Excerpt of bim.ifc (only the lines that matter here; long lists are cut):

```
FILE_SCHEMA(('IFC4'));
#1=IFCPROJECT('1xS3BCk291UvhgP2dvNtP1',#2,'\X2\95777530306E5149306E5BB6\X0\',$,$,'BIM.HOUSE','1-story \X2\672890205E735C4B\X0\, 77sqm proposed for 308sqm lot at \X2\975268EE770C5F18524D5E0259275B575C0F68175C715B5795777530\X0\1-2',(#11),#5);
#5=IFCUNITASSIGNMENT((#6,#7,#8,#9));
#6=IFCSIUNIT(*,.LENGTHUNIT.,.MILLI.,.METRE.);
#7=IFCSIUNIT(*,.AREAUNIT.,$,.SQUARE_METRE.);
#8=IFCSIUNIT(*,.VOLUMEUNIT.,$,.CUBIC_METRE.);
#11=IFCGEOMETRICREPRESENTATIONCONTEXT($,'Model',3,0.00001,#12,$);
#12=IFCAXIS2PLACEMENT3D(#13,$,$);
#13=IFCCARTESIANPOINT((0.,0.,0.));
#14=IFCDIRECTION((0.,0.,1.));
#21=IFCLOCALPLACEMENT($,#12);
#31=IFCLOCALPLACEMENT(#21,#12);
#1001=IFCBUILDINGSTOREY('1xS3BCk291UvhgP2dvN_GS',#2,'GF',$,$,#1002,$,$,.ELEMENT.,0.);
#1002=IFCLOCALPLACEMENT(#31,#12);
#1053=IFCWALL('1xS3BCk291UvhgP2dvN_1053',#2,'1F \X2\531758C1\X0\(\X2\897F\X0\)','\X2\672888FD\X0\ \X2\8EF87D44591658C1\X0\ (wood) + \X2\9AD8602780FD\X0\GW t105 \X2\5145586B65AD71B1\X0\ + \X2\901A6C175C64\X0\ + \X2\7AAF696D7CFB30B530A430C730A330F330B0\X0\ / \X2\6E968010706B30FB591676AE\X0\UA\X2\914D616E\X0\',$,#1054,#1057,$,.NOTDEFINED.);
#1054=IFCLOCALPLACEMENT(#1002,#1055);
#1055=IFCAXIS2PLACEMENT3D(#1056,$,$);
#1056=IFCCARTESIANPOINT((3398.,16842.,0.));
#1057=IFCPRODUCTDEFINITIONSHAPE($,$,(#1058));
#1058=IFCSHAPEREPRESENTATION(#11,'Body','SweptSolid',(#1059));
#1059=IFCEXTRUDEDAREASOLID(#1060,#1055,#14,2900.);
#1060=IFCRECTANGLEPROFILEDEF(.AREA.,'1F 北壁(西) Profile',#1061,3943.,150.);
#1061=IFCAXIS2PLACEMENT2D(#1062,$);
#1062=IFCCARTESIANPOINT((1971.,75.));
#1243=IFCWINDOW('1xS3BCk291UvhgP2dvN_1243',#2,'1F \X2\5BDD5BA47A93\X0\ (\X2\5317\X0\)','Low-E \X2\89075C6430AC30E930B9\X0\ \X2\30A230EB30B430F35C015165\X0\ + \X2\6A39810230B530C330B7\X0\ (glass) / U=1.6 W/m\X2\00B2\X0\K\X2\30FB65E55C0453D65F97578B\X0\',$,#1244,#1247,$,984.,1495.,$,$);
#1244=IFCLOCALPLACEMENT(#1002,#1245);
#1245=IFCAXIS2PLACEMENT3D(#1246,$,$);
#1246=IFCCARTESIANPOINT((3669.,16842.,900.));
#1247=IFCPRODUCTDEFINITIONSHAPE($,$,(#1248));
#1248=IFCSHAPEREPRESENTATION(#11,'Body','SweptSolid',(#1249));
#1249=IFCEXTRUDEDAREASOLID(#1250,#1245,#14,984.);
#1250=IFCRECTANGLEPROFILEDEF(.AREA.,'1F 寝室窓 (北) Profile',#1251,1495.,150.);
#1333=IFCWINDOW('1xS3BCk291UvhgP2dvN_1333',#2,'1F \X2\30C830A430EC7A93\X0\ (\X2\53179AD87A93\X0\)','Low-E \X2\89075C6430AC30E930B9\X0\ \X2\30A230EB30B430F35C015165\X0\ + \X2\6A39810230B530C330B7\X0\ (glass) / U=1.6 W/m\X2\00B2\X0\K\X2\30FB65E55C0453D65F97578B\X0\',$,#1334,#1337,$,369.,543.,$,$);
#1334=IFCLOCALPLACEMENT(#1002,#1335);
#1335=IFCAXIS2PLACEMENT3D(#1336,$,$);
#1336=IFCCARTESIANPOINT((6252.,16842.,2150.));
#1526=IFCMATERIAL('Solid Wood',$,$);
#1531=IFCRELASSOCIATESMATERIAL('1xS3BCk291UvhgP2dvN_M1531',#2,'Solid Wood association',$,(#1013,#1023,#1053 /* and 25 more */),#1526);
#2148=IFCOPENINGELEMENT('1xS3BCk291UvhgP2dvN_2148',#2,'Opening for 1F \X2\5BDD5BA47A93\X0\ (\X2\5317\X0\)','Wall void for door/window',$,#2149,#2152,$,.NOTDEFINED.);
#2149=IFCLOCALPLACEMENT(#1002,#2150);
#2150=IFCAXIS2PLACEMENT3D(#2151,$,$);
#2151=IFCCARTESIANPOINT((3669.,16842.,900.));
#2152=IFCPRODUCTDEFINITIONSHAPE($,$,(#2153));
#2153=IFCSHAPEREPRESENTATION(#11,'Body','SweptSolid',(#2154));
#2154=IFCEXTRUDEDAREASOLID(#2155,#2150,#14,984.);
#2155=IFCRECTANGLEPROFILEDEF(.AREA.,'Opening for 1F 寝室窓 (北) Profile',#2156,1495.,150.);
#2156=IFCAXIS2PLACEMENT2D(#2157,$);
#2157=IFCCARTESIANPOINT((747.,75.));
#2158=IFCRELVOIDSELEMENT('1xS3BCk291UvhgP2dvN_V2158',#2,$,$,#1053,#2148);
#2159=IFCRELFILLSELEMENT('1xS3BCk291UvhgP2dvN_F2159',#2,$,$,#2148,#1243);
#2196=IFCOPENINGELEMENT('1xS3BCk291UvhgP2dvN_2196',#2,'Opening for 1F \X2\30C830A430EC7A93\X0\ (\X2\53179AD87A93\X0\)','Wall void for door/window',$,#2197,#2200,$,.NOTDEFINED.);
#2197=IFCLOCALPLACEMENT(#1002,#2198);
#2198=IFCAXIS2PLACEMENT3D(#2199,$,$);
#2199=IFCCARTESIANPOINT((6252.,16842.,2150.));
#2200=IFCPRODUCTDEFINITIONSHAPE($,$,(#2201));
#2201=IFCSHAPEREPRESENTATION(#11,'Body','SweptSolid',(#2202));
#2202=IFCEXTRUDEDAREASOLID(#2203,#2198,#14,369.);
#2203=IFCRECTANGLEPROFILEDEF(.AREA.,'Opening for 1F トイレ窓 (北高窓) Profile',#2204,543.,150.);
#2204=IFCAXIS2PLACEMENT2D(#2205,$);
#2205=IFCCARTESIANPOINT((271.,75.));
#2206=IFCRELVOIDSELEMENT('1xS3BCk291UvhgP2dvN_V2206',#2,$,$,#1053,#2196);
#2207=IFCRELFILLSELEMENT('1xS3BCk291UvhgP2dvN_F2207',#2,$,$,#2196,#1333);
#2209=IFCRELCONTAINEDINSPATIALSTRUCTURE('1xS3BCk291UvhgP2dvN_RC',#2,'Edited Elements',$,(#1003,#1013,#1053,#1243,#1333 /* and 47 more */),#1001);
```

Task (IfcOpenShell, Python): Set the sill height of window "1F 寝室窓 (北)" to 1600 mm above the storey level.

```python
import numpy as np
import ifcopenshell
import ifcopenshell.api.geometry
import ifcopenshell.geom
import ifcopenshell.util.element
import ifcopenshell.util.placement
import ifcopenshell.util.shape
import ifcopenshell.util.unit

model = ifcopenshell.open("bim.ifc")
unit_scale = ifcopenshell.util.unit.calculate_unit_scale(model)

window = model.by_guid("1xS3BCk291UvhgP2dvN_1243")
opening = window.FillsVoids[0].RelatingOpeningElement
storey = ifcopenshell.util.element.get_container(window, ifc_class="IfcBuildingStorey")
level = ifcopenshell.util.placement.get_local_placement(storey.ObjectPlacement)[2, 3]

# The opening's origin need not be at the sill, so measure its lowest point.
shape = ifcopenshell.geom.create_shape(ifcopenshell.geom.settings(), opening)
bottom = ifcopenshell.util.shape.get_shape_bottom_elevation(shape, shape.geometry) / unit_scale
dz = level + 1.6 / unit_scale - bottom

shift = np.array([0.0, 0.0, dz])
# The window is not placed relative to its opening, so move both.
for product in (opening, window):
    matrix = ifcopenshell.util.placement.get_local_placement(product.ObjectPlacement)
    matrix[:3, 3] += shift
    ifcopenshell.api.geometry.edit_object_placement(model, product=product, matrix=matrix, is_si=False)

print(f"moved by {dz * unit_scale:+.3f} m")

model.write("bim_v2.ifc")
```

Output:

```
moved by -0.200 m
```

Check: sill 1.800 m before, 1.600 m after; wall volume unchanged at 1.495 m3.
